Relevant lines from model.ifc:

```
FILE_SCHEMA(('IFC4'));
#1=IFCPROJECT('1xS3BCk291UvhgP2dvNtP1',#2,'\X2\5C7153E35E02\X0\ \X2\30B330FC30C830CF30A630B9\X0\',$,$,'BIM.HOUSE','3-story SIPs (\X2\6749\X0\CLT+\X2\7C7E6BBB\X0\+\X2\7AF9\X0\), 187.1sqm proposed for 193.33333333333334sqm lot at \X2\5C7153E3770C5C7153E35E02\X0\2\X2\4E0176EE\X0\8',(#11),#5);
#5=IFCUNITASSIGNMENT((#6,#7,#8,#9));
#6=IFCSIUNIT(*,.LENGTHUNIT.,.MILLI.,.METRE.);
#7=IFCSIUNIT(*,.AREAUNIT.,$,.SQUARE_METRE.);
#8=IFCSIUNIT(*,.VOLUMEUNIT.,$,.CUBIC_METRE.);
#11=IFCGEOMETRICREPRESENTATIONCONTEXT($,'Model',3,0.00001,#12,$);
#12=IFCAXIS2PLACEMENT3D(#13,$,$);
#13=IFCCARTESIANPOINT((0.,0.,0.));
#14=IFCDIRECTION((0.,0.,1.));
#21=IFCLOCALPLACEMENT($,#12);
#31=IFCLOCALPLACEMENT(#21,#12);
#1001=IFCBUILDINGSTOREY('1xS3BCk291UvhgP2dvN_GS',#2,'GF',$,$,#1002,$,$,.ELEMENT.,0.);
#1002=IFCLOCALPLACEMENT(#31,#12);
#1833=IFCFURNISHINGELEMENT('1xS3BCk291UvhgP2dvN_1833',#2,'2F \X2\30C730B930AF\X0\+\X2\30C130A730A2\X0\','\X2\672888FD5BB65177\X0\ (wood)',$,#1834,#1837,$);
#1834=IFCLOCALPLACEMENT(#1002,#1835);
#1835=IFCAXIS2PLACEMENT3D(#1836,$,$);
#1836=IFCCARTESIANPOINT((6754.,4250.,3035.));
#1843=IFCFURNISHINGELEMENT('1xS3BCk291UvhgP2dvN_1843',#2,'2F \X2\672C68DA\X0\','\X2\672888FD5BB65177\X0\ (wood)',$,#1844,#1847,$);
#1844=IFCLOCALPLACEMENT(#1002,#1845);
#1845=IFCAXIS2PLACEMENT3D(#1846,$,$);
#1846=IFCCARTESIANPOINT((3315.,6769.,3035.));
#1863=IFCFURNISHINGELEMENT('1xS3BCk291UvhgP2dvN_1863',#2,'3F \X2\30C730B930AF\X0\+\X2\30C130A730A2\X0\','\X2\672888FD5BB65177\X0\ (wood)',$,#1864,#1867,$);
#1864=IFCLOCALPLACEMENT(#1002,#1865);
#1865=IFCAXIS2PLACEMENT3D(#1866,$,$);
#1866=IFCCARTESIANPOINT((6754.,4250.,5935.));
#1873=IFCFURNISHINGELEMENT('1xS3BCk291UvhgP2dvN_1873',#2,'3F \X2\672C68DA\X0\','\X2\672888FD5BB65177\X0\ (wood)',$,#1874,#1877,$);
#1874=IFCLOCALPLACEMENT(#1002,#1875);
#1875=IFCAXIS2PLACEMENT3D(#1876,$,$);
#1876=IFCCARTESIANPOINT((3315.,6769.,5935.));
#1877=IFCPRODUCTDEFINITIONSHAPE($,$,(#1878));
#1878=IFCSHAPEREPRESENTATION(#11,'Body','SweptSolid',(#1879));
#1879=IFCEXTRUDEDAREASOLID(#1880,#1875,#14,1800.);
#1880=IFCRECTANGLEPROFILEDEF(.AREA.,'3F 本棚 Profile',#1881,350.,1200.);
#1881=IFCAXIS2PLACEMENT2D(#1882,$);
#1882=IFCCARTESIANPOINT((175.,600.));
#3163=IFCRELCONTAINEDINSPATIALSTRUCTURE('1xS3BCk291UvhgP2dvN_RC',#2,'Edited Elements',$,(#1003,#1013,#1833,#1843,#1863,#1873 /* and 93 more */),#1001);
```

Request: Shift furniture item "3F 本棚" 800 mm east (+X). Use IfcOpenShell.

```python
import ifcopenshell
import ifcopenshell.api.geometry
import ifcopenshell.util.placement

model = ifcopenshell.open("model.ifc")

item = model.by_guid("1xS3BCk291UvhgP2dvN_1873")
matrix = ifcopenshell.util.placement.get_local_placement(item.ObjectPlacement)
matrix[0, 3] += 800.0
ifcopenshell.api.geometry.edit_object_placement(model, product=item, matrix=matrix, is_si=False)

print(ifcopenshell.util.placement.get_local_placement(item.ObjectPlacement).round(3) + 0.0)

model.write("model_rev.ifc")
```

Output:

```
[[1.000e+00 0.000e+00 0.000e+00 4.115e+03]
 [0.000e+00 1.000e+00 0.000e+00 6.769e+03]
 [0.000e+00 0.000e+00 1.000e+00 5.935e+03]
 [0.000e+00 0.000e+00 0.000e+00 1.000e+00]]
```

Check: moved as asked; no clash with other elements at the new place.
